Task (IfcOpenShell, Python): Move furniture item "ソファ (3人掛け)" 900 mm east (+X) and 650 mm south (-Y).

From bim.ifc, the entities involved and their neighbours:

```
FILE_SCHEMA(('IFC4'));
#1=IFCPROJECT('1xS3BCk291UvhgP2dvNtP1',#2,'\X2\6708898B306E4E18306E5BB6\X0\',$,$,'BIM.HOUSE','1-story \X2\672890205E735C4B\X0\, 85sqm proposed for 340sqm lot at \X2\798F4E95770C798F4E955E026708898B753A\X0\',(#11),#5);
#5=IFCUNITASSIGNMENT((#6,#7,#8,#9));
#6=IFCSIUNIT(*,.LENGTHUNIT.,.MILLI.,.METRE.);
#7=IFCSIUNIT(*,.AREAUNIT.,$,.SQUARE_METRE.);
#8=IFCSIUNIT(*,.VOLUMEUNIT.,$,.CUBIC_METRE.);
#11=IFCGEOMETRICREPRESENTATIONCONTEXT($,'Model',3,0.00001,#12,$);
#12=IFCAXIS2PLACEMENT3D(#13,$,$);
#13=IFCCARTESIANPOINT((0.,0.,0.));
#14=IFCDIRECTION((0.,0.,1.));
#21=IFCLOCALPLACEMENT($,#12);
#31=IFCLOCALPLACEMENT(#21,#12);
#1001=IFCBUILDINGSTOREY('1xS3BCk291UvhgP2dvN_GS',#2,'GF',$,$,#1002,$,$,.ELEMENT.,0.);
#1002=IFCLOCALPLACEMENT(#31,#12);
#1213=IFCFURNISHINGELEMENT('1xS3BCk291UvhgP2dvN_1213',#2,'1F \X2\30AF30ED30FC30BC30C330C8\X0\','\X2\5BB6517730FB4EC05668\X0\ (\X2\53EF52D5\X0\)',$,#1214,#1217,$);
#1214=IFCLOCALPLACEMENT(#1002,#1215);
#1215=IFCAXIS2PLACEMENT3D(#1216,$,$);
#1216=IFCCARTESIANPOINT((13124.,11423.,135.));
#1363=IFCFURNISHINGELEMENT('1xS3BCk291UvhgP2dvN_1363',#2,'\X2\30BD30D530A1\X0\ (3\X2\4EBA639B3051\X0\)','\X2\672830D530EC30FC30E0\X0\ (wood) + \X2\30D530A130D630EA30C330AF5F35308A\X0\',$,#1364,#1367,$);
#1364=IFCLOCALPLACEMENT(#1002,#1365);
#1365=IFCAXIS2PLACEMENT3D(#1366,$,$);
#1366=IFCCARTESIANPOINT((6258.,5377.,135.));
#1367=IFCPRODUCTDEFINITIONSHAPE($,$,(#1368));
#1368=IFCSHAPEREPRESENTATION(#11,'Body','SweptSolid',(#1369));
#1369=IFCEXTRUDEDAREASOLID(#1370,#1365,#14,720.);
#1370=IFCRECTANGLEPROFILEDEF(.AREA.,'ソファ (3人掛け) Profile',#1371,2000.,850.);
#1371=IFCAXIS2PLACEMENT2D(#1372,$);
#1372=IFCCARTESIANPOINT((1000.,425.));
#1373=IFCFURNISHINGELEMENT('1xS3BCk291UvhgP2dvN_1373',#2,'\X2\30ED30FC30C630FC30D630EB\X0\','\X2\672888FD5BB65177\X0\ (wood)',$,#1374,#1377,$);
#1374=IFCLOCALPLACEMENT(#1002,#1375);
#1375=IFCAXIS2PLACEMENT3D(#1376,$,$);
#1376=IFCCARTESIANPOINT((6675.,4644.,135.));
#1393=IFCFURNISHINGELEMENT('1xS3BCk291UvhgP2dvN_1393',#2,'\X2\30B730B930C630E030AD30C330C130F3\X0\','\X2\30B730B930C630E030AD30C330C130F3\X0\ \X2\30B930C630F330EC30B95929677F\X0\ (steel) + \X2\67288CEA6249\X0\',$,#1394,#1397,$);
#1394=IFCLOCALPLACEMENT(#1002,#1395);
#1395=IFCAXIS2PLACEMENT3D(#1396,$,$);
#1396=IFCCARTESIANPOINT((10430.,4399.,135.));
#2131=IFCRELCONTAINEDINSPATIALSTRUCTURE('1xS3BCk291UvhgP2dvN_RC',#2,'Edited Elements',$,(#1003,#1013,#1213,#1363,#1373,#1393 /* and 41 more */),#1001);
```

```python
import ifcopenshell
import ifcopenshell.api.geometry
import ifcopenshell.util.placement
import ifcopenshell.util.unit

model = ifcopenshell.open("bim.ifc")
unit_scale = ifcopenshell.util.unit.calculate_unit_scale(model)

item = model.by_guid("1xS3BCk291UvhgP2dvN_1363")
matrix = ifcopenshell.util.placement.get_local_placement(item.ObjectPlacement)
matrix[0, 3] += 0.9 / unit_scale
matrix[1, 3] -= 0.65 / unit_scale
ifcopenshell.api.geometry.edit_object_placement(model, product=item, matrix=matrix, is_si=False)

print(ifcopenshell.util.placement.get_local_placement(item.ObjectPlacement).round(3) + 0.0)

model.write("bim_updated.ifc")
```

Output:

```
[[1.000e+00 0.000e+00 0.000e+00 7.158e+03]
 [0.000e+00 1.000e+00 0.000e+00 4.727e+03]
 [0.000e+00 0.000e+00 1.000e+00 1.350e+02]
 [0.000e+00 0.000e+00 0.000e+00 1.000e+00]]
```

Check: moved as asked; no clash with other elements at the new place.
